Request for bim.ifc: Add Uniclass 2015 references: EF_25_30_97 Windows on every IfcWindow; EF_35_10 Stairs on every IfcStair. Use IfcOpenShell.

First a look at what the model holds.

```python
import ifcopenshell

model = ifcopenshell.open("bim.ifc")
print(model.schema)
print("classifications:", [c.Name for c in model.by_type("IfcClassification")])
for ifc_class in ("IfcDoor", "IfcRoof", "IfcStair", "IfcWall", "IfcWindow"):
    print(ifc_class, len(model.by_type(ifc_class)))
```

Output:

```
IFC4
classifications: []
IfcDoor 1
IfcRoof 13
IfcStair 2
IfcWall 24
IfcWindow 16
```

```python
import ifcopenshell
import ifcopenshell.api.classification

model = ifcopenshell.open("bim.ifc")

system = ifcopenshell.api.classification.add_classification(model, classification="Uniclass 2015")

codes = {
    "IfcWindow": ("EF_25_30_97", "Windows"),
    "IfcStair": ("EF_35_10", "Stairs"),
}
for ifc_class, (code, name) in codes.items():
    products = model.by_type(ifc_class)
    ifcopenshell.api.classification.add_reference(
        model, products=products, classification=system, identification=code, name=name
    )
    print(code, len(products))

model.write("bim_rev.ifc")
```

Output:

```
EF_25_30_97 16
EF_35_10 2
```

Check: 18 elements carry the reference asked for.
